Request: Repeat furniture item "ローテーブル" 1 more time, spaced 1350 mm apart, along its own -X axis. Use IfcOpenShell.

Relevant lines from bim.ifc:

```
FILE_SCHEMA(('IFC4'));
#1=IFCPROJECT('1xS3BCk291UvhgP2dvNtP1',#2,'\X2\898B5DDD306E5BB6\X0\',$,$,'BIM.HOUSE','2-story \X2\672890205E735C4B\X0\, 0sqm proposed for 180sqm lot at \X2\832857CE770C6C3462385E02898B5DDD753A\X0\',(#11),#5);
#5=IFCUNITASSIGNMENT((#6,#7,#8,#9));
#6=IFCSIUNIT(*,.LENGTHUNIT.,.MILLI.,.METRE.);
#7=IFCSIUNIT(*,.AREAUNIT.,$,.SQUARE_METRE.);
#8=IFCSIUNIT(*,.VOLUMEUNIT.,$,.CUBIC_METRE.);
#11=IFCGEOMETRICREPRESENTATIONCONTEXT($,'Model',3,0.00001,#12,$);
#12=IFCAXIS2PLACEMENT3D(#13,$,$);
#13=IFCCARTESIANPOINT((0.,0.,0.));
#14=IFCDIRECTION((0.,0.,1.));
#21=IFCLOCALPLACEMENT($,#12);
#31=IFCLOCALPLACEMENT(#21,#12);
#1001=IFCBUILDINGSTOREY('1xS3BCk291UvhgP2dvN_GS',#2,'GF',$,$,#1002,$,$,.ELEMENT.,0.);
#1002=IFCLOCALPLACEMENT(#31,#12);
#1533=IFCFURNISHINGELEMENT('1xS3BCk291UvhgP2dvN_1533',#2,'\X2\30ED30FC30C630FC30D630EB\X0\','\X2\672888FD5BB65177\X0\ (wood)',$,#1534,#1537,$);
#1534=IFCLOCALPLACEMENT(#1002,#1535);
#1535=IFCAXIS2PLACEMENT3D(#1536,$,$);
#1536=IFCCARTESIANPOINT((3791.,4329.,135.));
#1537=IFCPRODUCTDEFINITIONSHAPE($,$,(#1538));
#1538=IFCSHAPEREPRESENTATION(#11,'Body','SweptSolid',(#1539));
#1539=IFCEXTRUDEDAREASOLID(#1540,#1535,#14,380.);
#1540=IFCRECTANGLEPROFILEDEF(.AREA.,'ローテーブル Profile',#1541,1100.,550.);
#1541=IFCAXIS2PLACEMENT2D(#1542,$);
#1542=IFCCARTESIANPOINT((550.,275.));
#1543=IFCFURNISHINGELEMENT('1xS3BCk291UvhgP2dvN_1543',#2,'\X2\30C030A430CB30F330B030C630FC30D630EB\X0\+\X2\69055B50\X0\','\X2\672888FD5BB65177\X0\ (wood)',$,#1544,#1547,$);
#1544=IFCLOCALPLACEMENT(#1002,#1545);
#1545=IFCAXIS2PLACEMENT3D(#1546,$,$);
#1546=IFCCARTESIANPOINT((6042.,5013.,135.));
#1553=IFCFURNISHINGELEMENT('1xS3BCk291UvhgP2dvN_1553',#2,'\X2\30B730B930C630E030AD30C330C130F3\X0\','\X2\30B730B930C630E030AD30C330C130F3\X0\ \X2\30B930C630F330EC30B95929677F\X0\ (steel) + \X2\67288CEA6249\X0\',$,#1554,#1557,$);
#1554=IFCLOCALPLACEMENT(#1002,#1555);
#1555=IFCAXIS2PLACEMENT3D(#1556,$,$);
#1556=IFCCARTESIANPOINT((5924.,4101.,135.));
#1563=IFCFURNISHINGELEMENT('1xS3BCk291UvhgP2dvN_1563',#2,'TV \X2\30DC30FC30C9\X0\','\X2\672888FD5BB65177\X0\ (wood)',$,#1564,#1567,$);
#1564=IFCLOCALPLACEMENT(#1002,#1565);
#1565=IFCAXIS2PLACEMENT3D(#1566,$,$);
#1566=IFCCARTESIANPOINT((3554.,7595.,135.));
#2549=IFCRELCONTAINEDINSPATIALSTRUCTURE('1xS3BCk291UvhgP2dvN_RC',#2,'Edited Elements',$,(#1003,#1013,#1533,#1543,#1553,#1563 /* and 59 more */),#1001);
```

```python
import ifcopenshell
import ifcopenshell.api.geometry
import ifcopenshell.api.root
import ifcopenshell.util.element
import ifcopenshell.util.placement
import ifcopenshell.util.unit

model = ifcopenshell.open("bim.ifc")
unit_scale = ifcopenshell.util.unit.calculate_unit_scale(model)


def reuse_history(source, copy):
    """copy_class also copies each property set's owner history, people and application; keep the originals."""
    for rel in copy.IsDefinedBy:
        if rel.is_a("IfcRelDefinesByProperties") and (history := rel.RelatingPropertyDefinition.OwnerHistory):
            rel.RelatingPropertyDefinition.OwnerHistory = source.OwnerHistory
            ifcopenshell.util.element.remove_deep2(model, history)


source = model.by_guid("1xS3BCk291UvhgP2dvN_1533")
base = ifcopenshell.util.placement.get_local_placement(source.ObjectPlacement)
step = -base[:3, 0] * 1.35 / unit_scale

for i in range(1, 2):
    copy = ifcopenshell.api.root.copy_class(model, product=source)
    copy.Representation = ifcopenshell.util.element.copy_deep(
        model, source.Representation, exclude=["IfcGeometricRepresentationContext", "IfcRepresentationMap"]
    )
    reuse_history(source, copy)
    matrix = base.copy()
    matrix[:3, 3] += i * step
    print("added at", matrix[:3, 3].round(3) + 0.0)
    ifcopenshell.api.geometry.edit_object_placement(model, product=copy, matrix=matrix, is_si=False)

model.write("bim_updated.ifc")
```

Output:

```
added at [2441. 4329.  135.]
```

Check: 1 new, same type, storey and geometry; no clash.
